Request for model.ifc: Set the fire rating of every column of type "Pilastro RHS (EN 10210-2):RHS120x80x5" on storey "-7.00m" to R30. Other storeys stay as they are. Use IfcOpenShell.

First a look at what the model holds.

```python
import ifcopenshell
import ifcopenshell.util.element

model = ifcopenshell.open("model.ifc")
print(model.schema)
storey = next(s for s in model.by_type("IfcBuildingStorey") if s.Name == "-7.00m")
columns = [e for e in ifcopenshell.util.element.get_decomposition(storey) if e.is_a("IfcColumn")]
seen = {}
for e in columns:
    element_type = ifcopenshell.util.element.get_type(e)
    key = (element_type.Name if element_type != e and element_type else None, ifcopenshell.util.element.get_pset(e, "Pset_ColumnCommon", "FireRating"))
    seen[key] = seen.get(key, 0) + 1
for (name, value), count in sorted(seen.items(), key=str):
    print(count, "x", name, "|", value)
```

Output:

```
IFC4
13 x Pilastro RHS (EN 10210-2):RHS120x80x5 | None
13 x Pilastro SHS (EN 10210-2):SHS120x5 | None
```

```python
import ifcopenshell
import ifcopenshell.api.pset
import ifcopenshell.util.element

model = ifcopenshell.open("model.ifc")

storey = next(s for s in model.by_type("IfcBuildingStorey") if s.Name == "-7.00m")
columns = [e for e in ifcopenshell.util.element.get_decomposition(storey) if e.is_a("IfcColumn")]

count = 0
for e in columns:
    element_type = ifcopenshell.util.element.get_type(e)
    if element_type in (None, e) or element_type.Name != "Pilastro RHS (EN 10210-2):RHS120x80x5":
        continue
    # add_pset returns the element's existing set when there is one.
    pset = ifcopenshell.api.pset.add_pset(model, product=e, name="Pset_ColumnCommon")
    ifcopenshell.api.pset.edit_pset(model, pset=pset, properties={"FireRating": "R30"})
    count += 1

print(count, "columns updated")

model.write("model_rev.ifc")
```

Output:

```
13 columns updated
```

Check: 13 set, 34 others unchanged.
